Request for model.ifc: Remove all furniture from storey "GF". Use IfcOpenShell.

First a look at what the model holds.

```python
import ifcopenshell
import ifcopenshell.util.element

model = ifcopenshell.open("model.ifc")
print(model.schema)
storey = next(s for s in model.by_type("IfcBuildingStorey") if s.Name == "GF")
furniture = [e for e in ifcopenshell.util.element.get_decomposition(storey) if e.is_a("IfcFurnishingElement")]
seen = {}
for e in furniture:
    element_type = ifcopenshell.util.element.get_type(e)
    name = element_type.Name if element_type not in (None, e) else None
    seen[name] = seen.get(name, 0) + 1
for name, count in sorted(seen.items(), key=str):
    print(count, "x", name)
```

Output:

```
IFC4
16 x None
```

```python
import ifcopenshell
import ifcopenshell.api.root
import ifcopenshell.util.element

model = ifcopenshell.open("model.ifc")

storey = next(s for s in model.by_type("IfcBuildingStorey") if s.Name == "GF")
furniture = [e for e in ifcopenshell.util.element.get_decomposition(storey) if e.is_a("IfcFurnishingElement")]

for e in furniture:
    ifcopenshell.api.root.remove_product(model, product=e)
print(len(furniture), "removed")

model.write("model_v2.ifc")
```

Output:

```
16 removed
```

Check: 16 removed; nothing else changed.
